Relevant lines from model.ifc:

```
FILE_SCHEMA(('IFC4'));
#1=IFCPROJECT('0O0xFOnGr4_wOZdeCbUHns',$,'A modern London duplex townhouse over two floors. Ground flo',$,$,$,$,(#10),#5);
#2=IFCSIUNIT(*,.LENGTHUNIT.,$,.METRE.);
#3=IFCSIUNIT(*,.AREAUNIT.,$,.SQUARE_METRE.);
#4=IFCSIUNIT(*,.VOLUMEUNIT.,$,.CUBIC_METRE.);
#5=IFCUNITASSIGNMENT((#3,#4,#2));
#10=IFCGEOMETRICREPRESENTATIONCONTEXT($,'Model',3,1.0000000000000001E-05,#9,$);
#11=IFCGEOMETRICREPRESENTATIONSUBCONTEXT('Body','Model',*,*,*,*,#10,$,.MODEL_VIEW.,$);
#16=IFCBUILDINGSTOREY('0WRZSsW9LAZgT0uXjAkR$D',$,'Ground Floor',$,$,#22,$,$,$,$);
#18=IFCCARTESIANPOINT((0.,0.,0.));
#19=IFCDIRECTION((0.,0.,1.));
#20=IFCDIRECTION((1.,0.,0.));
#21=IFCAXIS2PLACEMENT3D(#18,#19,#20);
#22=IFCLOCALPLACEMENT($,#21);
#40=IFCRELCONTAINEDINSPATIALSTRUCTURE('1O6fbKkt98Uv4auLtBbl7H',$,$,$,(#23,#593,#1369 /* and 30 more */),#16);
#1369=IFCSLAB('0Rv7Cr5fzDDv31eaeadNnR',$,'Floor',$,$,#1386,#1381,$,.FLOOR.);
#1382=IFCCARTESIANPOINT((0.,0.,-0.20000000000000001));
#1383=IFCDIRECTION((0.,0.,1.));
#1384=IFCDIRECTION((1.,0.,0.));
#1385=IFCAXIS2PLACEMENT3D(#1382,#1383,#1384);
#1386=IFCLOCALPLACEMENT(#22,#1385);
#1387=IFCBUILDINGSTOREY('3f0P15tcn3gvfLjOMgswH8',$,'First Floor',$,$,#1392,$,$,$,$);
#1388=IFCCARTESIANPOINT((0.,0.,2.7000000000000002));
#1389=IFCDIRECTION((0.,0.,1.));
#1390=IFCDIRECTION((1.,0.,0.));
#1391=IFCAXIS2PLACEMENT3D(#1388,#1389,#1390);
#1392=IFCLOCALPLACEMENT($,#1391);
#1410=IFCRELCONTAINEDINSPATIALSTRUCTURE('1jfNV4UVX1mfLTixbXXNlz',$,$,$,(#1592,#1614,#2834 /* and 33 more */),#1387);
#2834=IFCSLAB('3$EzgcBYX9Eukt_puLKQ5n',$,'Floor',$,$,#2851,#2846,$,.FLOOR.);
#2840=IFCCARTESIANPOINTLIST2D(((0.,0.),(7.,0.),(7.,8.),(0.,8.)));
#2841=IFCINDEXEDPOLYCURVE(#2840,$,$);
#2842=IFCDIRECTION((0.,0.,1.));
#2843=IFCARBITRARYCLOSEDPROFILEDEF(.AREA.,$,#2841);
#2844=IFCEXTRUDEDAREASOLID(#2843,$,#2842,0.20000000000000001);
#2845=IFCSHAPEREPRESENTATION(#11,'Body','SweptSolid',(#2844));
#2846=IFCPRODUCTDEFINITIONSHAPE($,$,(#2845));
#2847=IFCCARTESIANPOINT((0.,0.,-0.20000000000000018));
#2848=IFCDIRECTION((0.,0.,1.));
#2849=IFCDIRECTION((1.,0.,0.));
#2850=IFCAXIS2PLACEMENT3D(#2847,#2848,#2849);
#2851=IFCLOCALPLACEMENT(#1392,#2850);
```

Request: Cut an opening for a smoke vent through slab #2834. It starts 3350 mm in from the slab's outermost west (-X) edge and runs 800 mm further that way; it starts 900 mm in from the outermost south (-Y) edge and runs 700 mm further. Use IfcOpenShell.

```python
import numpy as np
import ifcopenshell
import ifcopenshell.api.feature
import ifcopenshell.api.geometry
import ifcopenshell.api.root
import ifcopenshell.geom
import ifcopenshell.util.placement
import ifcopenshell.util.representation
import ifcopenshell.util.shape
import ifcopenshell.util.unit

model = ifcopenshell.open("model.ifc")
unit_scale = ifcopenshell.util.unit.calculate_unit_scale(model)
settings = ifcopenshell.geom.settings()


def volume(element):
    """Net volume in cubic metres, openings subtracted."""
    shape = ifcopenshell.geom.create_shape(settings, element)
    return ifcopenshell.util.shape.get_volume(shape.geometry)


slab = model.by_guid("3$EzgcBYX9Eukt_puLKQ5n")
before = volume(slab)

# Extent in the slab's own axes, in metres. The edges named are its -X and -Y sides.
slab_shape = ifcopenshell.geom.create_shape(settings, slab)
vertices = ifcopenshell.util.shape.get_vertices(slab_shape.geometry)
x_min, y_min, bottom = vertices.min(axis=0)
top = vertices[:, 2].max()

opening = ifcopenshell.api.root.create_entity(model, ifc_class="IfcOpeningElement", name="Smoke vent opening", predefined_type="OPENING")
context = ifcopenshell.util.representation.get_context(model, "Model", "Body", "MODEL_VIEW")
width, depth = 0.8, 0.7
outline = [(0.0, 0.0), (width, 0.0), (width, depth), (0.0, depth), (0.0, 0.0)]
# Overshoot both faces by 50 mm so the cut is clean.
shape = ifcopenshell.api.geometry.add_slab_representation(
    model, context=context, depth=top - bottom + 0.1, polyline=outline
)
ifcopenshell.api.geometry.assign_representation(model, product=opening, representation=shape)

matrix = ifcopenshell.util.placement.get_local_placement(slab.ObjectPlacement)
matrix[:, 3] = matrix @ np.append(np.array([x_min + 3.35, y_min + 0.9, bottom - 0.05]) / unit_scale, 1.0)
ifcopenshell.api.geometry.edit_object_placement(model, product=opening, matrix=matrix, is_si=False)
ifcopenshell.api.feature.add_feature(model, feature=opening, element=slab)

after = volume(slab)

print(f"slab volume {before:.3f} -> {after:.3f} m3")

model.write("model_updated.ifc")
```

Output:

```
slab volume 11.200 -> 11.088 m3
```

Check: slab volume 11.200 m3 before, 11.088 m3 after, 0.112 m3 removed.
